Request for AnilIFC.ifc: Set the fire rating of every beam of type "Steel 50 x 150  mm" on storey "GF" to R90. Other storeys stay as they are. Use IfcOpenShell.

First a look at what the model holds.

```python
import ifcopenshell
import ifcopenshell.util.element

model = ifcopenshell.open("AnilIFC.ifc")
print(model.schema)
storey = next(s for s in model.by_type("IfcBuildingStorey") if s.Name == "GF")
beams = [e for e in ifcopenshell.util.element.get_decomposition(storey) if e.is_a("IfcBeam")]
seen = {}
for e in beams:
    element_type = ifcopenshell.util.element.get_type(e)
    key = (element_type.Name if element_type != e and element_type else None, ifcopenshell.util.element.get_pset(e, "Pset_BeamCommon", "FireRating"))
    seen[key] = seen.get(key, 0) + 1
for (name, value), count in sorted(seen.items(), key=str):
    print(count, "x", name, "|", value)
```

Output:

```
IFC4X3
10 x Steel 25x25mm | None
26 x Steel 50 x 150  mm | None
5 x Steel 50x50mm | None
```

```python
import ifcopenshell
import ifcopenshell.api.pset
import ifcopenshell.util.element

model = ifcopenshell.open("AnilIFC.ifc")

storey = next(s for s in model.by_type("IfcBuildingStorey") if s.Name == "GF")
beams = [e for e in ifcopenshell.util.element.get_decomposition(storey) if e.is_a("IfcBeam")]

count = 0
for e in beams:
    element_type = ifcopenshell.util.element.get_type(e)
    if element_type in (None, e) or element_type.Name != "Steel 50 x 150  mm":
        continue
    # add_pset returns the element's existing set when there is one.
    pset = ifcopenshell.api.pset.add_pset(model, product=e, name="Pset_BeamCommon")
    ifcopenshell.api.pset.edit_pset(model, pset=pset, properties={"FireRating": "R90"})
    count += 1

print(count, "beams updated")

model.write("AnilIFC-out.ifc")
```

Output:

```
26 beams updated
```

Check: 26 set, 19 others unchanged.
